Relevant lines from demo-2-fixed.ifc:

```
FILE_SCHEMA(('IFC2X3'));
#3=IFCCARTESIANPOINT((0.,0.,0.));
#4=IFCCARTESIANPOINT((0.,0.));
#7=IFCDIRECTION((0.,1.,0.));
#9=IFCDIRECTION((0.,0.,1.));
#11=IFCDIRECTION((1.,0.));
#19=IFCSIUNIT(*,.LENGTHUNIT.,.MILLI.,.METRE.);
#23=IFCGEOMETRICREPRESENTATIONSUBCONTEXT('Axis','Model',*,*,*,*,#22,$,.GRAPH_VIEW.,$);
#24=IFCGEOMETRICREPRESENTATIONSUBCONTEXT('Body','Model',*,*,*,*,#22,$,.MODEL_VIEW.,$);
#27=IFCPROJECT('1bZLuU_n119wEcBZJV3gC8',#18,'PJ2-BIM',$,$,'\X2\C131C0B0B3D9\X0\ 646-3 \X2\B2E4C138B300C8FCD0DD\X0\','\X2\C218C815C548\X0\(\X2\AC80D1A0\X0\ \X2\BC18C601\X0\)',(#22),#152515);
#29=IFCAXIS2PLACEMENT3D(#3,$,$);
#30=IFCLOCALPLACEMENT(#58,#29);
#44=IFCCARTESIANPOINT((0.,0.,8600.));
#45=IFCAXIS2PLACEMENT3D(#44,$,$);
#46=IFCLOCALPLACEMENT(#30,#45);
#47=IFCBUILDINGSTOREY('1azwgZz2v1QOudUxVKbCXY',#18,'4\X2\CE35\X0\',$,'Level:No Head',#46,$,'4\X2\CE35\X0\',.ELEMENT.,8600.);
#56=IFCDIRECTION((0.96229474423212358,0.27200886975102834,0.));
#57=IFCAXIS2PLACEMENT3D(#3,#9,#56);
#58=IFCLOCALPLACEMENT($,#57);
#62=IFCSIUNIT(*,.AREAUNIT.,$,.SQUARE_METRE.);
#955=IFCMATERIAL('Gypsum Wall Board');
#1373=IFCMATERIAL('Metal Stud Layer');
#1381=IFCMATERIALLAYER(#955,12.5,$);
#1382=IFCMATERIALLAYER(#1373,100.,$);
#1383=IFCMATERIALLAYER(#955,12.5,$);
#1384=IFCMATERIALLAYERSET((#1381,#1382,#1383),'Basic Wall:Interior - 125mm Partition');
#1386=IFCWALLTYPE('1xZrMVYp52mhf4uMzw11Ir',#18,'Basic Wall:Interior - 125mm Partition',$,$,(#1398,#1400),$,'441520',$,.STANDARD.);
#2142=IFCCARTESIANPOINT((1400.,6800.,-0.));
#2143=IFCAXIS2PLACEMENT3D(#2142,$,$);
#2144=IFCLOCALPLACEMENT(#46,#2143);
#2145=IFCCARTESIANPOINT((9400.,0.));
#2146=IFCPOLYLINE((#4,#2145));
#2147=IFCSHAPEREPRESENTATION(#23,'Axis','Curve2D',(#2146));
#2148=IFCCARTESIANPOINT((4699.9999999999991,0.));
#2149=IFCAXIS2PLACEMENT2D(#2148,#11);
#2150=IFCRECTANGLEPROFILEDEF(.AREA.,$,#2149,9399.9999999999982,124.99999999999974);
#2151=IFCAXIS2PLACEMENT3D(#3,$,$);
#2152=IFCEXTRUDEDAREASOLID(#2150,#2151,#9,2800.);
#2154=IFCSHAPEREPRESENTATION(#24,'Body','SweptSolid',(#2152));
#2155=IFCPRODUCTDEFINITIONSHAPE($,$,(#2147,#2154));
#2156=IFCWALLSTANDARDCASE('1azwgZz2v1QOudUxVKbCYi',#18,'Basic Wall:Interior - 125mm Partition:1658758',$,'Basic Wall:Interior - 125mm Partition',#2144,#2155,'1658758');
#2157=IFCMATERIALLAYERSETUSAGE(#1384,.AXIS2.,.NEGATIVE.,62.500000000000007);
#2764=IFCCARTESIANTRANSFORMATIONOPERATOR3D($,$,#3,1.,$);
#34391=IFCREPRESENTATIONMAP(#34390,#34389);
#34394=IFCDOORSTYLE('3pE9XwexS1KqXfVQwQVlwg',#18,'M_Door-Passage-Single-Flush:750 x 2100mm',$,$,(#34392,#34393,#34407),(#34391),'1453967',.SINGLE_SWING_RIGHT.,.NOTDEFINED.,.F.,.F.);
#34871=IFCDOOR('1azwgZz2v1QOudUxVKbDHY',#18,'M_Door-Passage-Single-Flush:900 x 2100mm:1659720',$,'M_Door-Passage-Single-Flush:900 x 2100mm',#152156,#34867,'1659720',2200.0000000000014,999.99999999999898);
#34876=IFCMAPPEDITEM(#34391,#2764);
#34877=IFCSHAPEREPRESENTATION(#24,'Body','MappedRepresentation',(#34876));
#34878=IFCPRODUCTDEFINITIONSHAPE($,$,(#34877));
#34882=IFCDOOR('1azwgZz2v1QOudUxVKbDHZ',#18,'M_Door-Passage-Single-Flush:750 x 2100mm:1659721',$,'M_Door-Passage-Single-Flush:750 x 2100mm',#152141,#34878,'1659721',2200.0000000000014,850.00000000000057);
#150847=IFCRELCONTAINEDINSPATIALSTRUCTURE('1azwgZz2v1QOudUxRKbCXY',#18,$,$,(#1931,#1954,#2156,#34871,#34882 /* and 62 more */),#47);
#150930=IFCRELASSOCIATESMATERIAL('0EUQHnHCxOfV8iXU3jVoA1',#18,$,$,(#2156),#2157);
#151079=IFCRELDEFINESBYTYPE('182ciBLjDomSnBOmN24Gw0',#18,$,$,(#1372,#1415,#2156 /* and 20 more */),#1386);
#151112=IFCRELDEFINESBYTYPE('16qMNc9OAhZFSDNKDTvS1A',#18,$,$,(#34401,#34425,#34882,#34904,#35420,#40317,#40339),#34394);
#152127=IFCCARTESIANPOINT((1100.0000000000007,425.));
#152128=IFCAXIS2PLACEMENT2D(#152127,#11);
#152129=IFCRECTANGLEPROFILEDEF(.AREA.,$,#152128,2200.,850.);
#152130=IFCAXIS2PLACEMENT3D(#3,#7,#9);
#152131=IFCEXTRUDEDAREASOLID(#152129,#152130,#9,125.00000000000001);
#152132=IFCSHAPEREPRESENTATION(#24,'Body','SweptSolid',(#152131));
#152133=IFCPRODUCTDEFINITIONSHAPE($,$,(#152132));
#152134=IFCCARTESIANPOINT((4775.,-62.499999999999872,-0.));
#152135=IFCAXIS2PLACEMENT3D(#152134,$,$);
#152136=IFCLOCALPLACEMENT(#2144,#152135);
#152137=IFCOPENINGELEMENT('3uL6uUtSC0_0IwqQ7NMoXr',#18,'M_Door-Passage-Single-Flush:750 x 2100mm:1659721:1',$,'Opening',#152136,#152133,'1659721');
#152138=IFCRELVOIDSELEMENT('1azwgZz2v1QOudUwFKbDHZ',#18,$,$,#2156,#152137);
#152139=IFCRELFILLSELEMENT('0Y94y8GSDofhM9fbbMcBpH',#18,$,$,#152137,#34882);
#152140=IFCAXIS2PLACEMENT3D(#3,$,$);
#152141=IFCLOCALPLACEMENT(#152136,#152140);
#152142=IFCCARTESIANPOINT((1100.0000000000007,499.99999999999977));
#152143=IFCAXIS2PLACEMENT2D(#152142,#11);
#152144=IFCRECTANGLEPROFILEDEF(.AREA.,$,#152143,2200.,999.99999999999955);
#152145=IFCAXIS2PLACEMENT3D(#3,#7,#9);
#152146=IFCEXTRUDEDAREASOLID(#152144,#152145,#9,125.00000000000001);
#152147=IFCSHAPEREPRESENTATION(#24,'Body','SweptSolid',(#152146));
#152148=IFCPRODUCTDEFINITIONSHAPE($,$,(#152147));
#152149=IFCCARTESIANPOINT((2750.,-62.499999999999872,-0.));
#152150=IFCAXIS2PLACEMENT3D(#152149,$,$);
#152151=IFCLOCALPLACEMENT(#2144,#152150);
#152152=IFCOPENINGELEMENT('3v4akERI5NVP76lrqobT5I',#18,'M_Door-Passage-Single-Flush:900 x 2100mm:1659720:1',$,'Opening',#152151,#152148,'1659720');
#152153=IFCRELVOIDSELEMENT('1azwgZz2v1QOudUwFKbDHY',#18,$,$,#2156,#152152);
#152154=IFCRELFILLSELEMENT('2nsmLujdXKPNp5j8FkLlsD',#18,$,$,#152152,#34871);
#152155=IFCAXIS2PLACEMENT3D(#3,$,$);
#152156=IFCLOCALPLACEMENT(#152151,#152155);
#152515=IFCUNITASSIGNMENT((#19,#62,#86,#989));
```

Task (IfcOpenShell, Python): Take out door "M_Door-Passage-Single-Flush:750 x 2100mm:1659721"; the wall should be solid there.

```python
import ifcopenshell
import ifcopenshell.api.feature
import ifcopenshell.api.root
import ifcopenshell.geom
import ifcopenshell.util.shape

model = ifcopenshell.open("demo-2-fixed.ifc")
settings = ifcopenshell.geom.settings()


def volume(element):
    """Net volume in cubic metres, openings subtracted."""
    shape = ifcopenshell.geom.create_shape(settings, element)
    return ifcopenshell.util.shape.get_volume(shape.geometry)


door = model.by_guid("1azwgZz2v1QOudUxVKbDHZ")
opening = door.FillsVoids[0].RelatingOpeningElement
wall = opening.VoidsElements[0].RelatingBuildingElement
before = volume(wall)

ifcopenshell.api.root.remove_product(model, product=door)
ifcopenshell.api.feature.remove_feature(model, feature=opening)

after = volume(wall)

print(f"wall volume {before:.3f} -> {after:.3f} m3")

model.write("demo-2-fixed_edited.ifc")
```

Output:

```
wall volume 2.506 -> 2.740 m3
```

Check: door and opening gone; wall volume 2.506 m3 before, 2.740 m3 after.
